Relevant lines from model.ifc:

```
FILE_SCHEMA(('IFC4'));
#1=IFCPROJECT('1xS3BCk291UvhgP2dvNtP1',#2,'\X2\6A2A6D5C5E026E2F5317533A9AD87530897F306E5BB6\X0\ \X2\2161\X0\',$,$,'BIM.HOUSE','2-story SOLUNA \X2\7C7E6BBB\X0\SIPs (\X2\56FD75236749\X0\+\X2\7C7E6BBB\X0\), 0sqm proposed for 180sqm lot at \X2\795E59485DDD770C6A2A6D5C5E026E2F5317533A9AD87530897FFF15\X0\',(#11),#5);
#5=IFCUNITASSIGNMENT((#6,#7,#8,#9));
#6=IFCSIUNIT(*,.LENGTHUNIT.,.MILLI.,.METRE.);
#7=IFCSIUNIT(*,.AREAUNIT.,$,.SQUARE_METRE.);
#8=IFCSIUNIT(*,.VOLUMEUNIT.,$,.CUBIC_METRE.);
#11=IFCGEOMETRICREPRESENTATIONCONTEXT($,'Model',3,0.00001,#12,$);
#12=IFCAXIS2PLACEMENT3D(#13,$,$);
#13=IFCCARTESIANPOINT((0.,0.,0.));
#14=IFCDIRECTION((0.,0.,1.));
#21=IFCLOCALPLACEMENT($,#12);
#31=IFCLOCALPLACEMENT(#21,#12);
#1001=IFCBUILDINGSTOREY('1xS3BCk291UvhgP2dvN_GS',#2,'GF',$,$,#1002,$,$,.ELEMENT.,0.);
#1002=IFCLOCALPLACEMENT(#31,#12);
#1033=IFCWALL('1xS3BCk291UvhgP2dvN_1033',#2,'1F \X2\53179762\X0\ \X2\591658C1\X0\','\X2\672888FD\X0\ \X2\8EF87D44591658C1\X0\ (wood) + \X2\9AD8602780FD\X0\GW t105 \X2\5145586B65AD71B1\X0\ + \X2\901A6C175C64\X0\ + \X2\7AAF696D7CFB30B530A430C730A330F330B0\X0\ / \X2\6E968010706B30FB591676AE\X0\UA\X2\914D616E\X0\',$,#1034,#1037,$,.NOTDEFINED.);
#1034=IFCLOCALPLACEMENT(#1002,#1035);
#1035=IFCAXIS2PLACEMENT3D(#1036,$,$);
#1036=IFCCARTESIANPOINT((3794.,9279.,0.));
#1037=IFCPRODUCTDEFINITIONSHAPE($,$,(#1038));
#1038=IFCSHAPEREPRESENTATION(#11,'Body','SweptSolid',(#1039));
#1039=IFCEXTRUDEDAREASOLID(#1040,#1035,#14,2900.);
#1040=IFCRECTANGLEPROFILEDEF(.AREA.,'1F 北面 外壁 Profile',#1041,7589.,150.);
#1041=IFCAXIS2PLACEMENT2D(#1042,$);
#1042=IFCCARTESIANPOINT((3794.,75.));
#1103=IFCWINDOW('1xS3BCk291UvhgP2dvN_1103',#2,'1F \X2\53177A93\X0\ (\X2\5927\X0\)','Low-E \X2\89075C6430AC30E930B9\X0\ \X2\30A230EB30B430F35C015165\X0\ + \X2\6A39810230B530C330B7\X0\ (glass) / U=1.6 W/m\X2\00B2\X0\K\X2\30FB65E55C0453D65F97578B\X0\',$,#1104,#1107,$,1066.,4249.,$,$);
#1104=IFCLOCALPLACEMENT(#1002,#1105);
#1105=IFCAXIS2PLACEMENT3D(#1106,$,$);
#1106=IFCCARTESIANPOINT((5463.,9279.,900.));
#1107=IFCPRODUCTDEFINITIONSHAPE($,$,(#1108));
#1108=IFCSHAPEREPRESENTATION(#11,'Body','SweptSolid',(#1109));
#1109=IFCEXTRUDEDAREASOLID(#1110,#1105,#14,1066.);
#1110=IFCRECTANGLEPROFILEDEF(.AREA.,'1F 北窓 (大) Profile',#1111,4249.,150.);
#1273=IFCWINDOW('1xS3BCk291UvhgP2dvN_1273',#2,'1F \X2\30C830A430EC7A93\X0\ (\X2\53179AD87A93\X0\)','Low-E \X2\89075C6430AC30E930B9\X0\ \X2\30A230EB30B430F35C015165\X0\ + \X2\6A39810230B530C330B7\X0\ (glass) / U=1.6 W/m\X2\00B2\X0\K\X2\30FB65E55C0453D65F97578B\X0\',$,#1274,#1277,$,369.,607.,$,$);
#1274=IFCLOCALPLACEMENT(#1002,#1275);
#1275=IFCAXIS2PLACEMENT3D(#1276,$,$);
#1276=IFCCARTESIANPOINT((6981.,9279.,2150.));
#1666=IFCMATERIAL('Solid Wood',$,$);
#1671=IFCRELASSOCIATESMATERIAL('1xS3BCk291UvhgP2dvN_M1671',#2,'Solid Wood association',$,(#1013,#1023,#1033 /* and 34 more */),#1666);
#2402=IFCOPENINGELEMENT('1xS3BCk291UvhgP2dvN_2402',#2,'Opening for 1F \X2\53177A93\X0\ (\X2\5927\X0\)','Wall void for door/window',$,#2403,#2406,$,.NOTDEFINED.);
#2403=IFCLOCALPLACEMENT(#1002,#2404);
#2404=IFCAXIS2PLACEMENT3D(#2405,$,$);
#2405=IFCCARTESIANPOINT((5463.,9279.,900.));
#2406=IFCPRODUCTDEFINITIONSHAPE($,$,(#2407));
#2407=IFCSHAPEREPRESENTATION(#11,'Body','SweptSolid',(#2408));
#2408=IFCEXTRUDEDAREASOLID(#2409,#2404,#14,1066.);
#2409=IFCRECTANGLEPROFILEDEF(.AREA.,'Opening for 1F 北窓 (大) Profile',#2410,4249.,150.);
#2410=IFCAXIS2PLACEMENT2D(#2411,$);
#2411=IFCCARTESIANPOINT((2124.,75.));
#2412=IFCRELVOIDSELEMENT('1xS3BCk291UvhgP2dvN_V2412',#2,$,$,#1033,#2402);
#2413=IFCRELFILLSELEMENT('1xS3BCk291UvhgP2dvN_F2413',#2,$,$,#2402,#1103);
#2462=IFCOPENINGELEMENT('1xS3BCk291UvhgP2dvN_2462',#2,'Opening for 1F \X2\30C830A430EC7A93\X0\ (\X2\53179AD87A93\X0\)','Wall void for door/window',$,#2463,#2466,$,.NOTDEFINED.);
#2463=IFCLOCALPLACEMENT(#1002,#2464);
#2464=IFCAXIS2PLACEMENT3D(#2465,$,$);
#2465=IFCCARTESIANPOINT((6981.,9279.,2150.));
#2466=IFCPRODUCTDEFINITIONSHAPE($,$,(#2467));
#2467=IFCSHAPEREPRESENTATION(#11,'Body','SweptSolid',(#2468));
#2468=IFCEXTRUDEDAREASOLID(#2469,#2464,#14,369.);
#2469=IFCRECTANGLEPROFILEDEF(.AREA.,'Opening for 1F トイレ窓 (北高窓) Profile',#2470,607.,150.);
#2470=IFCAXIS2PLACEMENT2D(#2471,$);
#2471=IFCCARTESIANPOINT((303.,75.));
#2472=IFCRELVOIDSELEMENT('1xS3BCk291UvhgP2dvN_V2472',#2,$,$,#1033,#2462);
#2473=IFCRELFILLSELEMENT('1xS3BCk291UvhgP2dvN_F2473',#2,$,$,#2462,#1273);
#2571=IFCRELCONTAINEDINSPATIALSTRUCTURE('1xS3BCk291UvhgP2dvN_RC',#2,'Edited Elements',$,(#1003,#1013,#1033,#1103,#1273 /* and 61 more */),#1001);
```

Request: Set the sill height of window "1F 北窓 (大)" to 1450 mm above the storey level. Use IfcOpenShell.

```python
import numpy as np
import ifcopenshell
import ifcopenshell.api.geometry
import ifcopenshell.geom
import ifcopenshell.util.element
import ifcopenshell.util.placement
import ifcopenshell.util.shape
import ifcopenshell.util.unit

model = ifcopenshell.open("model.ifc")
unit_scale = ifcopenshell.util.unit.calculate_unit_scale(model)

window = model.by_guid("1xS3BCk291UvhgP2dvN_1103")
opening = window.FillsVoids[0].RelatingOpeningElement
storey = ifcopenshell.util.element.get_container(window, ifc_class="IfcBuildingStorey")
level = ifcopenshell.util.placement.get_local_placement(storey.ObjectPlacement)[2, 3]

# The opening's origin need not be at the sill, so measure its lowest point.
shape = ifcopenshell.geom.create_shape(ifcopenshell.geom.settings(), opening)
bottom = ifcopenshell.util.shape.get_shape_bottom_elevation(shape, shape.geometry) / unit_scale
dz = level + 1.45 / unit_scale - bottom

shift = np.array([0.0, 0.0, dz])
# The window is not placed relative to its opening, so move both.
for product in (opening, window):
    matrix = ifcopenshell.util.placement.get_local_placement(product.ObjectPlacement)
    matrix[:3, 3] += shift
    ifcopenshell.api.geometry.edit_object_placement(model, product=product, matrix=matrix, is_si=False)

print(f"moved by {dz * unit_scale:+.3f} m")

model.write("model_edited.ifc")
```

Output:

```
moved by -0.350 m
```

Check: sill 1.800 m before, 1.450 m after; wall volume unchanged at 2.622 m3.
